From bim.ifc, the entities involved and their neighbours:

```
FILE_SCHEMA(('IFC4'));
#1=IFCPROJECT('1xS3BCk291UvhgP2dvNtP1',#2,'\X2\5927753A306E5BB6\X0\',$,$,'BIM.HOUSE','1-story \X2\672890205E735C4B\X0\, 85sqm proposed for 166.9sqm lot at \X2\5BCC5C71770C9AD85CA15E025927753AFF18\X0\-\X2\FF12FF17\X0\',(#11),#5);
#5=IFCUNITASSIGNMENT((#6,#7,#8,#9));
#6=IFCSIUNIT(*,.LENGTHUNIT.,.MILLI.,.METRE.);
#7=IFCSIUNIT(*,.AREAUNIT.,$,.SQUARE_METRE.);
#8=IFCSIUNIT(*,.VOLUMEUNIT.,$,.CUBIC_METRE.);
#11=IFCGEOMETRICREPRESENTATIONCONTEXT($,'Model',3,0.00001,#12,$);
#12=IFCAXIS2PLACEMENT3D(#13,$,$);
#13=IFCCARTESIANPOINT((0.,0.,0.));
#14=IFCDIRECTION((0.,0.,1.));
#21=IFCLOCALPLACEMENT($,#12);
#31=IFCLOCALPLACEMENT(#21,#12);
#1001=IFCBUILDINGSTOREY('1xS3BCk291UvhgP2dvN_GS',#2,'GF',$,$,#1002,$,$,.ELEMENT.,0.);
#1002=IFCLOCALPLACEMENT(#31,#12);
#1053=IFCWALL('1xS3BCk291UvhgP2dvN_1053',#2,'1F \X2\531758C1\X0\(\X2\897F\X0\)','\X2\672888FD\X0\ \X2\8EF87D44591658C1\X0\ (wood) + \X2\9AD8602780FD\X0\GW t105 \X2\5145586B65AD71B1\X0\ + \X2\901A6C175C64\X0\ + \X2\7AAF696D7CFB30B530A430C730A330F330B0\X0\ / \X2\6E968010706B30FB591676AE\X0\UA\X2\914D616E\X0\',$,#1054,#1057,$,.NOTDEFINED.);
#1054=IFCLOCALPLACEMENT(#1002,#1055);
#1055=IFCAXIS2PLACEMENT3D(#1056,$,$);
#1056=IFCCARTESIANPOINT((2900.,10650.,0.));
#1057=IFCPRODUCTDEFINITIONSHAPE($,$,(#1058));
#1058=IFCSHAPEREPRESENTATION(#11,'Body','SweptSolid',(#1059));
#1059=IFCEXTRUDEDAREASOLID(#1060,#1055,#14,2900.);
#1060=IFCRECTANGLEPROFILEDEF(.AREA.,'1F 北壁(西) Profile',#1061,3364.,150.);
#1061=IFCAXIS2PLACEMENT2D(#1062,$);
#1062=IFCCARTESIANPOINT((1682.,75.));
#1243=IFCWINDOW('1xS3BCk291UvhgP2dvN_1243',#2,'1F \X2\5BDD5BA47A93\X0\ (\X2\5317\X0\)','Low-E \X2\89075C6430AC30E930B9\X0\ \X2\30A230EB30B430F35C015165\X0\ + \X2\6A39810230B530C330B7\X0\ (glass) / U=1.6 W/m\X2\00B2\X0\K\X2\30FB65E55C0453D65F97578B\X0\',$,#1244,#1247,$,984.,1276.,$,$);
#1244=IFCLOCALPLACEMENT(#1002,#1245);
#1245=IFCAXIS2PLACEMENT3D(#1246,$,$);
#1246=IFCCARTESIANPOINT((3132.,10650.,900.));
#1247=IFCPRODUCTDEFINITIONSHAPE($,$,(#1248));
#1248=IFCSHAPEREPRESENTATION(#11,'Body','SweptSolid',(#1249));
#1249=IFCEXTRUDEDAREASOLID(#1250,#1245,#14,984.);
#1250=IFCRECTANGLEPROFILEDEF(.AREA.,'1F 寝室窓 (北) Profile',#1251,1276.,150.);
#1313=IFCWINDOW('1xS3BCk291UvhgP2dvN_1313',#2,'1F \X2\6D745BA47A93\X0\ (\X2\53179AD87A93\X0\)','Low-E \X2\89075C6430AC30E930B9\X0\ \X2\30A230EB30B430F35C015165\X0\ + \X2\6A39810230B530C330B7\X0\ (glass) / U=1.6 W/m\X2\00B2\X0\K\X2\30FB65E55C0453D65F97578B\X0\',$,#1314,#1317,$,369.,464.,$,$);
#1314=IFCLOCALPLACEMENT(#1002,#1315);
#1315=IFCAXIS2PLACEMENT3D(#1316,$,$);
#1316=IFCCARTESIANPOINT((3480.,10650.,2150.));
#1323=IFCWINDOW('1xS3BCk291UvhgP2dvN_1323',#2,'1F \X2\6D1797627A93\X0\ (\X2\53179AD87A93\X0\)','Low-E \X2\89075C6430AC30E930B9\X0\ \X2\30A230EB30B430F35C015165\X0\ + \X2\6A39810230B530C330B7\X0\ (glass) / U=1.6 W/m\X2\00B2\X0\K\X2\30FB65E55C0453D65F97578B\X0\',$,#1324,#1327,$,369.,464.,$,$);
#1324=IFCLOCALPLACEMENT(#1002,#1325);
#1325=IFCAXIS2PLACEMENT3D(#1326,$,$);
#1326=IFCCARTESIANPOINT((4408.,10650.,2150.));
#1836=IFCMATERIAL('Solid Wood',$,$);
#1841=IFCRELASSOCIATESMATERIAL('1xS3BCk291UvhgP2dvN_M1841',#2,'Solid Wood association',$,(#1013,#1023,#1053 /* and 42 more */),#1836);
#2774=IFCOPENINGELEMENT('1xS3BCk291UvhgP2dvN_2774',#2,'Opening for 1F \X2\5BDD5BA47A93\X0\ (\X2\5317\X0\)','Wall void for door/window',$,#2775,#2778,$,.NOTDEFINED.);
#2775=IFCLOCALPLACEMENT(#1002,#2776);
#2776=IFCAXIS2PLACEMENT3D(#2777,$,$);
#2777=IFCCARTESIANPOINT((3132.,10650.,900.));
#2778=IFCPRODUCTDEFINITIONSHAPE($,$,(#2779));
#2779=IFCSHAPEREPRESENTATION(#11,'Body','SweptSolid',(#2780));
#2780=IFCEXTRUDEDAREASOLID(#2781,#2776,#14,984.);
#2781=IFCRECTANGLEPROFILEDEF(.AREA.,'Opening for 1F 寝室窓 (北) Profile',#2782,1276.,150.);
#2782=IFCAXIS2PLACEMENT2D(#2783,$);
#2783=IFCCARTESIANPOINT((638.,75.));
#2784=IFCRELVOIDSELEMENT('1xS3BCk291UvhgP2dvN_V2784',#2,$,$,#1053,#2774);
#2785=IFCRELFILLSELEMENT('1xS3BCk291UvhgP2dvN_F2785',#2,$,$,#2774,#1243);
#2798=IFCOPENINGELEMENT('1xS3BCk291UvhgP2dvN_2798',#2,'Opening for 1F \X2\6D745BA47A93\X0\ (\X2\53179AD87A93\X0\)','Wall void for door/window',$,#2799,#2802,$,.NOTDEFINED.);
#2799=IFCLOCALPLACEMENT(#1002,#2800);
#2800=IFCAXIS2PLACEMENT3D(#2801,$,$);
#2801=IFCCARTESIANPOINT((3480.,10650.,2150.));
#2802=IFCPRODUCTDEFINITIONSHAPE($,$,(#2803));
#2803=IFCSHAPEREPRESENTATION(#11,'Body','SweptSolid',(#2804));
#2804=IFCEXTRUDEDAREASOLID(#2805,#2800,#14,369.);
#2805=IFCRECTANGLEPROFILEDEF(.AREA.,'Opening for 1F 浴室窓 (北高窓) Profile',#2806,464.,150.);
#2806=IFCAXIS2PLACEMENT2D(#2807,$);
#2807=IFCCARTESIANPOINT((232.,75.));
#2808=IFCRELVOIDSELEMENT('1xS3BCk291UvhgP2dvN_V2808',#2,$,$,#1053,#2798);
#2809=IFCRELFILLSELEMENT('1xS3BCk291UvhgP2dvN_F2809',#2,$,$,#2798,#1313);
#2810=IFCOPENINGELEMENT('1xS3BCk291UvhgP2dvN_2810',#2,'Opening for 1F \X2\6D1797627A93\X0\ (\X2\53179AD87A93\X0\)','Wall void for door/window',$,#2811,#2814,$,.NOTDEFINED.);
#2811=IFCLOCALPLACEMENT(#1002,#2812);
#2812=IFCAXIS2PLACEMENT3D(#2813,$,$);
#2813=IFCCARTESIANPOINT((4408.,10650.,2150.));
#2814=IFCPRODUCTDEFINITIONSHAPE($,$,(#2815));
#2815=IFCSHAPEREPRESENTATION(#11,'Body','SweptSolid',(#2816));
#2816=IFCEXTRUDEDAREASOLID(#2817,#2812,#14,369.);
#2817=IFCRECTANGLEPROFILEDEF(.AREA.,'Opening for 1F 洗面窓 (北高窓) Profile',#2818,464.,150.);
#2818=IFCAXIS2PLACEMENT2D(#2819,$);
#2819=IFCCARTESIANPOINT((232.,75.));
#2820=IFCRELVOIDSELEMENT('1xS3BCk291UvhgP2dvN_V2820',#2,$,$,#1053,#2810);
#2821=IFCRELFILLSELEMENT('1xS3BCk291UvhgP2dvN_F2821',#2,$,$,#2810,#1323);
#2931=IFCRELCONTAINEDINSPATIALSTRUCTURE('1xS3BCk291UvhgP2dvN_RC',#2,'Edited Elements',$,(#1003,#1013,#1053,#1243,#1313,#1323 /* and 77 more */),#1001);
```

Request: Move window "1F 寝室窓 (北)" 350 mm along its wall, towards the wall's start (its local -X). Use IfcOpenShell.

```python
import ifcopenshell
import ifcopenshell.api.geometry
import ifcopenshell.util.placement
import ifcopenshell.util.unit

model = ifcopenshell.open("bim.ifc")
unit_scale = ifcopenshell.util.unit.calculate_unit_scale(model)

window = model.by_guid("1xS3BCk291UvhgP2dvN_1243")
opening = window.FillsVoids[0].RelatingOpeningElement
wall = opening.VoidsElements[0].RelatingBuildingElement

wall_matrix = ifcopenshell.util.placement.get_local_placement(wall.ObjectPlacement)
shift = wall_matrix[:3, 0] * -0.35 / unit_scale
before = ifcopenshell.util.placement.get_local_placement(window.ObjectPlacement)[:3, 3].copy()

# The window is not placed relative to its opening, so move both.
for product in (opening, window):
    matrix = ifcopenshell.util.placement.get_local_placement(product.ObjectPlacement)
    matrix[:3, 3] += shift
    ifcopenshell.api.geometry.edit_object_placement(model, product=product, matrix=matrix, is_si=False)

after = ifcopenshell.util.placement.get_local_placement(window.ObjectPlacement)[:3, 3]
print("window moved by", (after - before).round(3) + 0.0)

model.write("bim-out.ifc")
```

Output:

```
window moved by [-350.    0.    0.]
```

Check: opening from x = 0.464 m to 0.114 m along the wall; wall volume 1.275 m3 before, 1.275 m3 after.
